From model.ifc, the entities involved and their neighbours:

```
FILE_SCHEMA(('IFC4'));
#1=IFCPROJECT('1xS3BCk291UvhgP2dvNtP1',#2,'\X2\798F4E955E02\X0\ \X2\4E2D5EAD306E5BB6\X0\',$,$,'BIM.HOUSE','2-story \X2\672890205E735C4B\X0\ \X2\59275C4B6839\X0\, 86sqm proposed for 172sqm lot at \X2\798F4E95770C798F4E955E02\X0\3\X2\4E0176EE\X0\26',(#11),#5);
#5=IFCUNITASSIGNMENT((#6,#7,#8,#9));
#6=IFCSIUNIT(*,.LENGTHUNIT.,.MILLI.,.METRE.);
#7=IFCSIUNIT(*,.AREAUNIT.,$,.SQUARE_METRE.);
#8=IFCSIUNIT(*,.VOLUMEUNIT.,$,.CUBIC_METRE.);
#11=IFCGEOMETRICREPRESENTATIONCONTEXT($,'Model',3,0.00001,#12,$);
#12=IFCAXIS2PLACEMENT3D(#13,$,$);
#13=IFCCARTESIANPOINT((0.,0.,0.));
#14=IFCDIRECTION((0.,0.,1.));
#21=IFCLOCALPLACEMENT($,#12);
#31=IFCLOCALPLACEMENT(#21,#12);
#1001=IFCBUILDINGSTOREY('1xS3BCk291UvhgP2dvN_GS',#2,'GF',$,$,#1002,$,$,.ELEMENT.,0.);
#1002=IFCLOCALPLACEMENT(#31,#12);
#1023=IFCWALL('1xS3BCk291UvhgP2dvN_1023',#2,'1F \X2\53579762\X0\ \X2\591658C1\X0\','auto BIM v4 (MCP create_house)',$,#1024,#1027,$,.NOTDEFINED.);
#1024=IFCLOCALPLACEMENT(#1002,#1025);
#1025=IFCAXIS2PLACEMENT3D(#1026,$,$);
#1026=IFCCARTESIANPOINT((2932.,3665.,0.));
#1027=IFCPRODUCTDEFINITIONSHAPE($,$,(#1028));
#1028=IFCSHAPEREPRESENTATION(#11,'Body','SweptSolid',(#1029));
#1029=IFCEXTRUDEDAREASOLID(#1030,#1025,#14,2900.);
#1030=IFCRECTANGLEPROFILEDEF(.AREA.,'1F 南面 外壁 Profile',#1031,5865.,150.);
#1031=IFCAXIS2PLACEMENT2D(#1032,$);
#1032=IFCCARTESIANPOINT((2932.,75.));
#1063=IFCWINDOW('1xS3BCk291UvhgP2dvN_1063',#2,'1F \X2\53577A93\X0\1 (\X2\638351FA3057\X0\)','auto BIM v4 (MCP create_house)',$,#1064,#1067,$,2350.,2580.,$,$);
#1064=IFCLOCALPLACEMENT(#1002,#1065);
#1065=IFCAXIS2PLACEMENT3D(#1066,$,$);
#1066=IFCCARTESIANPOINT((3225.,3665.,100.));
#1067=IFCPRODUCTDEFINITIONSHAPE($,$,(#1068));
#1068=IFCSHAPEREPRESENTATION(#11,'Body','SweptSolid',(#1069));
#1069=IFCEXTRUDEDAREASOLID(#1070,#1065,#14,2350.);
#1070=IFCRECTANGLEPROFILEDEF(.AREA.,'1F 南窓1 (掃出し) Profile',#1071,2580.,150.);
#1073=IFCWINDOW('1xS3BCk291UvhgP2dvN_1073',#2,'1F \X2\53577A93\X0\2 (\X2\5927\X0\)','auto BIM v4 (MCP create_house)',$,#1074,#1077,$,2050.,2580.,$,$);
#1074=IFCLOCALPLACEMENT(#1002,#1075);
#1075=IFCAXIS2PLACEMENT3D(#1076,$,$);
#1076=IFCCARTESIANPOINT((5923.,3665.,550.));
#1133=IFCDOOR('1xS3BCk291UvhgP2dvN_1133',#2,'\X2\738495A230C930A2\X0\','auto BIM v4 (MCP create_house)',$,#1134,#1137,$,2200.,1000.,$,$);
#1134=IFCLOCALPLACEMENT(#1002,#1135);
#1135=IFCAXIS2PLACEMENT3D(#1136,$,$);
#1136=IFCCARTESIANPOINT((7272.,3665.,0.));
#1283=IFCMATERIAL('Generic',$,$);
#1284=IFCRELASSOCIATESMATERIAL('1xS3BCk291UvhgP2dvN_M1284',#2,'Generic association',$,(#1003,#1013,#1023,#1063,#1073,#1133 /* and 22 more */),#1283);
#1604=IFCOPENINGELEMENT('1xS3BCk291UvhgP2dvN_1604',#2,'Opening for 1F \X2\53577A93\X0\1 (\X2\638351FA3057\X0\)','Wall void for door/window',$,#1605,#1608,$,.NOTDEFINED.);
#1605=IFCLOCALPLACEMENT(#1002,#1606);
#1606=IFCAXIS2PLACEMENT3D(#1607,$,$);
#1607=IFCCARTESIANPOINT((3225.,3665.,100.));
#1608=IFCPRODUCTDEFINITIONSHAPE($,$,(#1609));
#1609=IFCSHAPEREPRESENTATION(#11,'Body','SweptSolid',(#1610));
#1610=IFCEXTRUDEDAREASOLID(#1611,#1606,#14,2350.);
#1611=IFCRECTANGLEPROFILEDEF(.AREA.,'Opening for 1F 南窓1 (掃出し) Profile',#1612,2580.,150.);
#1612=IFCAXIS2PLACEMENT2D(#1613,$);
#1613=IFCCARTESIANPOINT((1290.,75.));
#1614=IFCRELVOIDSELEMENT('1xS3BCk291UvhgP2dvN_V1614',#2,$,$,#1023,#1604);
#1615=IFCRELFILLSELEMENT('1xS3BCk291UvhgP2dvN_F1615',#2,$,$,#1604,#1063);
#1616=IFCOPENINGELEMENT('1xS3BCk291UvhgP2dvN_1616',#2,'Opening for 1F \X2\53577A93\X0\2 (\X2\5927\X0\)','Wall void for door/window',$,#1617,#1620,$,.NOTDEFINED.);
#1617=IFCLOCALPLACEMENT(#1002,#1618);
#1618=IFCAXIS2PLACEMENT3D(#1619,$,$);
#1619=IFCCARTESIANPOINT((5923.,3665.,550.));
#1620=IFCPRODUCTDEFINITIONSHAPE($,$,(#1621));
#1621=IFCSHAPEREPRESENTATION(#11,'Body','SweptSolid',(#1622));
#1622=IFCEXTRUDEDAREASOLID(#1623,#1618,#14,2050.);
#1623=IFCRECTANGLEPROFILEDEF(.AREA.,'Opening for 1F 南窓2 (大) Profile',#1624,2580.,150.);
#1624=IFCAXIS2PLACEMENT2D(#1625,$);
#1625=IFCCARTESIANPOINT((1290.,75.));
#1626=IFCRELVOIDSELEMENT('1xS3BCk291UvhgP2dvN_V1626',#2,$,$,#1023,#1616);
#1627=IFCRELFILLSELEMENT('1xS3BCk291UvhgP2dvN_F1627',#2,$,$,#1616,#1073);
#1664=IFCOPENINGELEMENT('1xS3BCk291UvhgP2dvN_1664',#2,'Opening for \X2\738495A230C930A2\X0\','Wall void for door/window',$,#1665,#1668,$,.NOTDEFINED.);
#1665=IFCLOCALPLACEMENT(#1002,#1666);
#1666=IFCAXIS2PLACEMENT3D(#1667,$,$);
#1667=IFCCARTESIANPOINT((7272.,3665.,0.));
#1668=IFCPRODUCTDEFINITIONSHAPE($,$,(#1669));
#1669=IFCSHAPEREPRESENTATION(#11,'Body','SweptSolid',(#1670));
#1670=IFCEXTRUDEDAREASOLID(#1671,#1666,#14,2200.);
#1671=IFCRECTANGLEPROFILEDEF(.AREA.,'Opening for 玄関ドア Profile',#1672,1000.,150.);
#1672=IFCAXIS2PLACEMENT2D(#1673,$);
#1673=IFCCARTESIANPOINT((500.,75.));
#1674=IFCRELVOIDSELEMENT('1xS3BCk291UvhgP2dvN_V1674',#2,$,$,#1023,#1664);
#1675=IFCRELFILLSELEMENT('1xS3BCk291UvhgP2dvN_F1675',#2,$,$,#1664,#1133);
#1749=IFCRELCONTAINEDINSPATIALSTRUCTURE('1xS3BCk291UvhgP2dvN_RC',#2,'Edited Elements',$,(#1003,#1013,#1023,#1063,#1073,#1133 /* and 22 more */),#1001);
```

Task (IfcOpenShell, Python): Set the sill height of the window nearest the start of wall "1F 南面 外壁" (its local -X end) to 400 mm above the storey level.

```python
import numpy as np
import ifcopenshell
import ifcopenshell.api.geometry
import ifcopenshell.geom
import ifcopenshell.util.element
import ifcopenshell.util.placement
import ifcopenshell.util.shape
import ifcopenshell.util.unit

model = ifcopenshell.open("model.ifc")
unit_scale = ifcopenshell.util.unit.calculate_unit_scale(model)

window = model.by_id(1063)
opening = window.FillsVoids[0].RelatingOpeningElement
storey = ifcopenshell.util.element.get_container(window, ifc_class="IfcBuildingStorey")
level = ifcopenshell.util.placement.get_local_placement(storey.ObjectPlacement)[2, 3]

# The opening's origin need not be at the sill, so measure its lowest point.
shape = ifcopenshell.geom.create_shape(ifcopenshell.geom.settings(), opening)
bottom = ifcopenshell.util.shape.get_shape_bottom_elevation(shape, shape.geometry) / unit_scale
dz = level + 0.4 / unit_scale - bottom

shift = np.array([0.0, 0.0, dz])
# The window is not placed relative to its opening, so move both.
for product in (opening, window):
    matrix = ifcopenshell.util.placement.get_local_placement(product.ObjectPlacement)
    matrix[:3, 3] += shift
    ifcopenshell.api.geometry.edit_object_placement(model, product=product, matrix=matrix, is_si=False)

print(f"moved by {dz * unit_scale:+.3f} m")

model.write("model-out.ifc")
```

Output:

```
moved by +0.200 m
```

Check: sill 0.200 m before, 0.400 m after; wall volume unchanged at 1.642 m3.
